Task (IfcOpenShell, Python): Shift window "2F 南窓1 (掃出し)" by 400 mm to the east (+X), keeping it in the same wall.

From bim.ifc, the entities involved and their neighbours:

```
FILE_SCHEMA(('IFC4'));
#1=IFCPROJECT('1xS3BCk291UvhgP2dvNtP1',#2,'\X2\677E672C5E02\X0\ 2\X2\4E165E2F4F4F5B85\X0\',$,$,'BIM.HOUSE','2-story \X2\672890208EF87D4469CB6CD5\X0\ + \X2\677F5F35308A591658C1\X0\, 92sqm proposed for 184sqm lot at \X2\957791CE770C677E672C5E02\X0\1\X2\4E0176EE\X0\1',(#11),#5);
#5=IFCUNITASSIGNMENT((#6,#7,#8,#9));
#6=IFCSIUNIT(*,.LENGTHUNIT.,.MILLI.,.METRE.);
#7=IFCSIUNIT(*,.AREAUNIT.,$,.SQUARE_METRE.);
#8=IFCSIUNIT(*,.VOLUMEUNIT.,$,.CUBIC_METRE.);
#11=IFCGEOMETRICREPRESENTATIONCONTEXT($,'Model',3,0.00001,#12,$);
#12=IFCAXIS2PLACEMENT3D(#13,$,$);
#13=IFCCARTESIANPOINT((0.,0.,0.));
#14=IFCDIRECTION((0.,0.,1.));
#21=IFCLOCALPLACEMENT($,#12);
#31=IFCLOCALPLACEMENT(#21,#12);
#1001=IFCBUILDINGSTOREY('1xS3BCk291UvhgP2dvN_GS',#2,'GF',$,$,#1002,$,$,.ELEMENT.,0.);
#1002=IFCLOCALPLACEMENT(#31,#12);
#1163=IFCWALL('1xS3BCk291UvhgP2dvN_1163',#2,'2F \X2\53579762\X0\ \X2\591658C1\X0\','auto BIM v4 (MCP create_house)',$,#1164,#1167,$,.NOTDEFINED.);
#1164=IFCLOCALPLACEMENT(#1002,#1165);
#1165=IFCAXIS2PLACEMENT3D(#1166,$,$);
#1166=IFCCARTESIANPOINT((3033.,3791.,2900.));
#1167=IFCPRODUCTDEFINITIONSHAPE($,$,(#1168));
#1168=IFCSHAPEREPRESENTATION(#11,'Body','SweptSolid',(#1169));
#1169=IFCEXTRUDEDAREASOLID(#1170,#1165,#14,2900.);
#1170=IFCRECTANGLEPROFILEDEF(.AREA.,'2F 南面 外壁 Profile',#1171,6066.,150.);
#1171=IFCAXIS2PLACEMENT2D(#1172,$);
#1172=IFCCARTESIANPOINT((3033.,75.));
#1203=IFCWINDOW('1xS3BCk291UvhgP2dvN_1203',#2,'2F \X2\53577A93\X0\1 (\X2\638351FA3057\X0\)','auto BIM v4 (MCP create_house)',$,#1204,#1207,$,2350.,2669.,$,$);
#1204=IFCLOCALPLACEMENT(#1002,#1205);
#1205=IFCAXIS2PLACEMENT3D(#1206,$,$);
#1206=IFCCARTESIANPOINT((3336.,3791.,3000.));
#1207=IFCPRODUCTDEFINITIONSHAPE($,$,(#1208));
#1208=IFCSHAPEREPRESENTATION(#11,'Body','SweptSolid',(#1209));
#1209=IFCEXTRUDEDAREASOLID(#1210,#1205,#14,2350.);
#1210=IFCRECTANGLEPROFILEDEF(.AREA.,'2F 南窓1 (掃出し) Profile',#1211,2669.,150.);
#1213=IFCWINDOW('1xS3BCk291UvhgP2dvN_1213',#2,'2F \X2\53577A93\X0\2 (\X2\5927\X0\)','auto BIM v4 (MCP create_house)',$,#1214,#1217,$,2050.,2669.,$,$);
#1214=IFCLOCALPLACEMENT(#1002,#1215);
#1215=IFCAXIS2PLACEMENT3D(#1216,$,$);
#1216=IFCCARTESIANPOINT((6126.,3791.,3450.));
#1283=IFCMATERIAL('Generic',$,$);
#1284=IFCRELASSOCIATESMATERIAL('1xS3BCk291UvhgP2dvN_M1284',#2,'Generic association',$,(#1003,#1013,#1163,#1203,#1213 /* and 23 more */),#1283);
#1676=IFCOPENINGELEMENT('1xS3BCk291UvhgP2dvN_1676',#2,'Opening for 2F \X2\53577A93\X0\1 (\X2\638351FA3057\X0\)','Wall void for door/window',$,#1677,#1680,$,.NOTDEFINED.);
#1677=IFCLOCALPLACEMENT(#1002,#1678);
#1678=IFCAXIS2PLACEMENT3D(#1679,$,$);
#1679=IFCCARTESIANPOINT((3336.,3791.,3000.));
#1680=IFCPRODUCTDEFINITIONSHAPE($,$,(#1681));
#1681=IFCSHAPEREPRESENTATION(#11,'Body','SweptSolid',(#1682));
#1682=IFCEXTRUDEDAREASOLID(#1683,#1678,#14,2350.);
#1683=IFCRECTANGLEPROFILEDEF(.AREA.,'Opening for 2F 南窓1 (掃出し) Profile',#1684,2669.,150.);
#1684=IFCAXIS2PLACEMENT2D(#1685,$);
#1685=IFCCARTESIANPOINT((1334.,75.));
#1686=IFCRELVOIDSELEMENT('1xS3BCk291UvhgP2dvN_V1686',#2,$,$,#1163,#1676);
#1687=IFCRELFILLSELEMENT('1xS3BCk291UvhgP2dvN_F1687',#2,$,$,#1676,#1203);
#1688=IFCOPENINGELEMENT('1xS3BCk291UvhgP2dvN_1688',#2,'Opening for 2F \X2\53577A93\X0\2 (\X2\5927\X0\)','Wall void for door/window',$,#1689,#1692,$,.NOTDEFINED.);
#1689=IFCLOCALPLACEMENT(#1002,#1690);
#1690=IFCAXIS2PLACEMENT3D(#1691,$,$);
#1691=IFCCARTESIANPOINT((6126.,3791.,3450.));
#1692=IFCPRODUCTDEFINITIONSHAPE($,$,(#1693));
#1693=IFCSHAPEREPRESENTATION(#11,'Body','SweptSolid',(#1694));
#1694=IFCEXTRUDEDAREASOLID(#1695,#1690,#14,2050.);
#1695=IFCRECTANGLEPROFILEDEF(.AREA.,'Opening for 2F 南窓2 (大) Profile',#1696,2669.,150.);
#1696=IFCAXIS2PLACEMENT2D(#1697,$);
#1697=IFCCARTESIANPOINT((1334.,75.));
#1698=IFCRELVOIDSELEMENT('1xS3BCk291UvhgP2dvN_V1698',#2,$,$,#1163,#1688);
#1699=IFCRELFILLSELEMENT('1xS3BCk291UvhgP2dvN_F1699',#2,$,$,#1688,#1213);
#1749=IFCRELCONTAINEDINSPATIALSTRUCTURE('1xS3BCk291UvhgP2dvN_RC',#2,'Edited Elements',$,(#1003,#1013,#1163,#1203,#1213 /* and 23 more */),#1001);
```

```python
import ifcopenshell
import ifcopenshell.api.geometry
import ifcopenshell.util.placement
import ifcopenshell.util.unit

model = ifcopenshell.open("bim.ifc")
unit_scale = ifcopenshell.util.unit.calculate_unit_scale(model)

window = model.by_id(1203)
opening = window.FillsVoids[0].RelatingOpeningElement
wall = opening.VoidsElements[0].RelatingBuildingElement

wall_matrix = ifcopenshell.util.placement.get_local_placement(wall.ObjectPlacement)
shift = wall_matrix[:3, 0] * 0.4 / unit_scale
before = ifcopenshell.util.placement.get_local_placement(window.ObjectPlacement)[:3, 3].copy()

# The window is not placed relative to its opening, so move both.
for product in (opening, window):
    matrix = ifcopenshell.util.placement.get_local_placement(product.ObjectPlacement)
    matrix[:3, 3] += shift
    ifcopenshell.api.geometry.edit_object_placement(model, product=product, matrix=matrix, is_si=False)

after = ifcopenshell.util.placement.get_local_placement(window.ObjectPlacement)[:3, 3]
print("window moved by", (after - before).round(3) + 0.0)

model.write("bim_rev.ifc")
```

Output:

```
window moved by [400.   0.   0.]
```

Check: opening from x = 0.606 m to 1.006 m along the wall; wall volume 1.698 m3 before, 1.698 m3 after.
